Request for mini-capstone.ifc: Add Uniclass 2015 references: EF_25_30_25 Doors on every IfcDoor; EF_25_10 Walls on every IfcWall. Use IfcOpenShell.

First a look at what the model holds.

```python
import ifcopenshell

model = ifcopenshell.open("mini-capstone.ifc")
print(model.schema)
print("classifications:", [c.Name for c in model.by_type("IfcClassification")])
for ifc_class in ("IfcDoor", "IfcRoof", "IfcStair", "IfcWall", "IfcWindow"):
    print(ifc_class, len(model.by_type(ifc_class)))
```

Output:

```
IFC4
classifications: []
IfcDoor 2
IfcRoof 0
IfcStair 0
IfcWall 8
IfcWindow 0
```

```python
import ifcopenshell
import ifcopenshell.api.classification

model = ifcopenshell.open("mini-capstone.ifc")

system = ifcopenshell.api.classification.add_classification(model, classification="Uniclass 2015")

codes = {
    "IfcDoor": ("EF_25_30_25", "Doors"),
    "IfcWall": ("EF_25_10", "Walls"),
}
for ifc_class, (code, name) in codes.items():
    products = model.by_type(ifc_class)
    ifcopenshell.api.classification.add_reference(
        model, products=products, classification=system, identification=code, name=name
    )
    print(code, len(products))

model.write("mini-capstone_updated.ifc")
```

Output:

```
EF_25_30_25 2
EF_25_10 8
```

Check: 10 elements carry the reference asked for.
